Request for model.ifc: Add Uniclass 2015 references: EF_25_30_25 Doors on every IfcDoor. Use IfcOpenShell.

First a look at what the model holds.

```python
import ifcopenshell

model = ifcopenshell.open("model.ifc")
print(model.schema)
print("classifications:", [c.Name for c in model.by_type("IfcClassification")])
for ifc_class in ("IfcDoor", "IfcRoof", "IfcStair", "IfcWall", "IfcWindow"):
    print(ifc_class, len(model.by_type(ifc_class)))
```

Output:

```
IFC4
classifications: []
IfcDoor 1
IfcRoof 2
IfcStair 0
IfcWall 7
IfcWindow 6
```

```python
import ifcopenshell
import ifcopenshell.api.classification

model = ifcopenshell.open("model.ifc")

system = ifcopenshell.api.classification.add_classification(model, classification="Uniclass 2015")

codes = {
    "IfcDoor": ("EF_25_30_25", "Doors"),
}
for ifc_class, (code, name) in codes.items():
    products = model.by_type(ifc_class)
    ifcopenshell.api.classification.add_reference(
        model, products=products, classification=system, identification=code, name=name
    )
    print(code, len(products))

model.write("model_v2.ifc")
```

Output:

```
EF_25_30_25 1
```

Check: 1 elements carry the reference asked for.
